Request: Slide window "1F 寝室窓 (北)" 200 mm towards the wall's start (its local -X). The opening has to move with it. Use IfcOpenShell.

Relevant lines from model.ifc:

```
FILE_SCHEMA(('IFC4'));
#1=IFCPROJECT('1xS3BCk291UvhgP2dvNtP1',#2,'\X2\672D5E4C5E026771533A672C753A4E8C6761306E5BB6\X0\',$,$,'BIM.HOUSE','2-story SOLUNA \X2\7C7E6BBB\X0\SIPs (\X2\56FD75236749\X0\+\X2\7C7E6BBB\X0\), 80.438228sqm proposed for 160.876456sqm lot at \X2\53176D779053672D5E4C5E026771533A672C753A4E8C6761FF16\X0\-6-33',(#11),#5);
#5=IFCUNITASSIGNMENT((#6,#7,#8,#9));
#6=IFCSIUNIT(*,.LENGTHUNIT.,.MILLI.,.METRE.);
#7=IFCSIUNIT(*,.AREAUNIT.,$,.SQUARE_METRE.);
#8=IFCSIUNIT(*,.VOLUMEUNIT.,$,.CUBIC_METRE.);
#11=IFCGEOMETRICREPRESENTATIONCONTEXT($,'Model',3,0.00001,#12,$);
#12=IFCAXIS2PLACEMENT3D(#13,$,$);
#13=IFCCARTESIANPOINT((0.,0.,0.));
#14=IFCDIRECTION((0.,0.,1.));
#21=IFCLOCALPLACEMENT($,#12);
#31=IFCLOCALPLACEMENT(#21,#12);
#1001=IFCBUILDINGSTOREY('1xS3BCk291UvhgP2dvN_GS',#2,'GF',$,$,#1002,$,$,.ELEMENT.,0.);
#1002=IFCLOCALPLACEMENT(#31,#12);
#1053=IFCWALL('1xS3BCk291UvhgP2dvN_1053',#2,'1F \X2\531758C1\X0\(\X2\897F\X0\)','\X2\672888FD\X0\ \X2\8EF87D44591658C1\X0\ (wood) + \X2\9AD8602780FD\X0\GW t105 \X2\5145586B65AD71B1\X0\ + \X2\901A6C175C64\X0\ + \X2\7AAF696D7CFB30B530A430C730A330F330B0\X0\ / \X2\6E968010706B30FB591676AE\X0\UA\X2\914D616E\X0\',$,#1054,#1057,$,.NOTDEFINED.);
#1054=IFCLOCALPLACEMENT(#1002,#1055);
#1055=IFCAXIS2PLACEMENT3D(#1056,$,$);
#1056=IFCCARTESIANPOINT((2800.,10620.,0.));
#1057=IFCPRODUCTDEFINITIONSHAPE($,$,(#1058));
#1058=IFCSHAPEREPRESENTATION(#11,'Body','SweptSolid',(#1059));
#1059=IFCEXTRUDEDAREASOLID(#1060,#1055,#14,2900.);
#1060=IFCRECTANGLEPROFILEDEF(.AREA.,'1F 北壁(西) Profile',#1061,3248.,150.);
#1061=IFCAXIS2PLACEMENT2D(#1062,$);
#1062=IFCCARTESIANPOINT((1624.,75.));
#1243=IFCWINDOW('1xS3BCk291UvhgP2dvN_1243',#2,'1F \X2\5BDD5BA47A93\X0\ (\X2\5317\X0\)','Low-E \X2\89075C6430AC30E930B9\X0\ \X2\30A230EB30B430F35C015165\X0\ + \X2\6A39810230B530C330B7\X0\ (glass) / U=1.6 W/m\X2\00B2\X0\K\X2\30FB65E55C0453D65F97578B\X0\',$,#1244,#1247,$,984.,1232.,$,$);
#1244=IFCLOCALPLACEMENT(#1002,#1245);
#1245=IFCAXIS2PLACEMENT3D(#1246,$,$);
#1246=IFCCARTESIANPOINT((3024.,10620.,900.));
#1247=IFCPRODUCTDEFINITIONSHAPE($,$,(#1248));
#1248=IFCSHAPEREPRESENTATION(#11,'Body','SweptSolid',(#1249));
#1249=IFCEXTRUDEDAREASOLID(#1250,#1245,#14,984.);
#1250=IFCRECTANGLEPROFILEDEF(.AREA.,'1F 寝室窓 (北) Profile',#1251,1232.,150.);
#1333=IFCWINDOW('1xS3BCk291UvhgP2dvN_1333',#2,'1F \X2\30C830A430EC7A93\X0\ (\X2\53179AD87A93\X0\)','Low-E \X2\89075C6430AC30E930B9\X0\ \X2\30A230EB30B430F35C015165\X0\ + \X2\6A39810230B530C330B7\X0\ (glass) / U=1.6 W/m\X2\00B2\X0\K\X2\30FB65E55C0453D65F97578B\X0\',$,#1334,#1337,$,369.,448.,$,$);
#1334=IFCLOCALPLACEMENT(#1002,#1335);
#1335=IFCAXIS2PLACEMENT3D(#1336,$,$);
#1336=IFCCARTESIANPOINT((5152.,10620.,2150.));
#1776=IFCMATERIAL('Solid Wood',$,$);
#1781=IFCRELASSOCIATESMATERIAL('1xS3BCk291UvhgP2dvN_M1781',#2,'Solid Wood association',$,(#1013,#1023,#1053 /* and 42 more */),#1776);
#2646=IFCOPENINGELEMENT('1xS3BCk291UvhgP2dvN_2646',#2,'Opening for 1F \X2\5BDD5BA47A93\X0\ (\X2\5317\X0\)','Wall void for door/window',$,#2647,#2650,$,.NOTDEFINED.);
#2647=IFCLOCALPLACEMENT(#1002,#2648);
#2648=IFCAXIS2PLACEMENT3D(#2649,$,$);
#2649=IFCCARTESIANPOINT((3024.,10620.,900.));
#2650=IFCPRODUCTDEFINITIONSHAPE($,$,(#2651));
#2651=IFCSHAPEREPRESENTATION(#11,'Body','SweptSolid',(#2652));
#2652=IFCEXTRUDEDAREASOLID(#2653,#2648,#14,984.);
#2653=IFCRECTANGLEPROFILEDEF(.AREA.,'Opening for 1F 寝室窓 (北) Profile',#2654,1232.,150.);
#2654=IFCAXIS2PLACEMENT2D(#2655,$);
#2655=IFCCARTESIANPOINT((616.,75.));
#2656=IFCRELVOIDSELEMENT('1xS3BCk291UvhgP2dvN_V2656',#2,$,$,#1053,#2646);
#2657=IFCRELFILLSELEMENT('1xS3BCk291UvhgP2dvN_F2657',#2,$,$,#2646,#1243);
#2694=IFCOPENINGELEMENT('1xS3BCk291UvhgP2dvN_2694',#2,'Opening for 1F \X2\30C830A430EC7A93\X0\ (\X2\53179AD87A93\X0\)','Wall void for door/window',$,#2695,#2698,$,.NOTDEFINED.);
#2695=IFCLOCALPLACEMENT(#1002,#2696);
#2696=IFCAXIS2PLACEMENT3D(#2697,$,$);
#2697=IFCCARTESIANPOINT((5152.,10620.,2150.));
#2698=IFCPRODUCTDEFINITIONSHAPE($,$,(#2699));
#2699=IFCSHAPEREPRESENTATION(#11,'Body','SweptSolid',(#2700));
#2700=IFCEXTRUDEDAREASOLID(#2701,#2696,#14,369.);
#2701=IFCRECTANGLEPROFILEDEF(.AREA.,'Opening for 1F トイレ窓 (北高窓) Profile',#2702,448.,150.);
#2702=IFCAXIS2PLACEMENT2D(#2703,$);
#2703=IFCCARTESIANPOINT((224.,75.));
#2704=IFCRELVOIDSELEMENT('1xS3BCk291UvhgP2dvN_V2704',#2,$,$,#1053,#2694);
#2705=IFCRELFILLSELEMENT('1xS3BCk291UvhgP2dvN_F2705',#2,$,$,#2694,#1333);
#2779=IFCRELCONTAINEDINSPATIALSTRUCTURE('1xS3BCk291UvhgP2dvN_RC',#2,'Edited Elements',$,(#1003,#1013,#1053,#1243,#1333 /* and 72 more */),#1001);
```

```python
import ifcopenshell
import ifcopenshell.api.geometry
import ifcopenshell.util.placement
import ifcopenshell.util.unit

model = ifcopenshell.open("model.ifc")
unit_scale = ifcopenshell.util.unit.calculate_unit_scale(model)

window = model.by_id(1243)
opening = window.FillsVoids[0].RelatingOpeningElement
wall = opening.VoidsElements[0].RelatingBuildingElement

wall_matrix = ifcopenshell.util.placement.get_local_placement(wall.ObjectPlacement)
shift = wall_matrix[:3, 0] * -0.2 / unit_scale
before = ifcopenshell.util.placement.get_local_placement(window.ObjectPlacement)[:3, 3].copy()

# The window is not placed relative to its opening, so move both.
for product in (opening, window):
    matrix = ifcopenshell.util.placement.get_local_placement(product.ObjectPlacement)
    matrix[:3, 3] += shift
    ifcopenshell.api.geometry.edit_object_placement(model, product=product, matrix=matrix, is_si=False)

after = ifcopenshell.util.placement.get_local_placement(window.ObjectPlacement)[:3, 3]
print("window moved by", (after - before).round(3) + 0.0)

model.write("model_updated.ifc")
```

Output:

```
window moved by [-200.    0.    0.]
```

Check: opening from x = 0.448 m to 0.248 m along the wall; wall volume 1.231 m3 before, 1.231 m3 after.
